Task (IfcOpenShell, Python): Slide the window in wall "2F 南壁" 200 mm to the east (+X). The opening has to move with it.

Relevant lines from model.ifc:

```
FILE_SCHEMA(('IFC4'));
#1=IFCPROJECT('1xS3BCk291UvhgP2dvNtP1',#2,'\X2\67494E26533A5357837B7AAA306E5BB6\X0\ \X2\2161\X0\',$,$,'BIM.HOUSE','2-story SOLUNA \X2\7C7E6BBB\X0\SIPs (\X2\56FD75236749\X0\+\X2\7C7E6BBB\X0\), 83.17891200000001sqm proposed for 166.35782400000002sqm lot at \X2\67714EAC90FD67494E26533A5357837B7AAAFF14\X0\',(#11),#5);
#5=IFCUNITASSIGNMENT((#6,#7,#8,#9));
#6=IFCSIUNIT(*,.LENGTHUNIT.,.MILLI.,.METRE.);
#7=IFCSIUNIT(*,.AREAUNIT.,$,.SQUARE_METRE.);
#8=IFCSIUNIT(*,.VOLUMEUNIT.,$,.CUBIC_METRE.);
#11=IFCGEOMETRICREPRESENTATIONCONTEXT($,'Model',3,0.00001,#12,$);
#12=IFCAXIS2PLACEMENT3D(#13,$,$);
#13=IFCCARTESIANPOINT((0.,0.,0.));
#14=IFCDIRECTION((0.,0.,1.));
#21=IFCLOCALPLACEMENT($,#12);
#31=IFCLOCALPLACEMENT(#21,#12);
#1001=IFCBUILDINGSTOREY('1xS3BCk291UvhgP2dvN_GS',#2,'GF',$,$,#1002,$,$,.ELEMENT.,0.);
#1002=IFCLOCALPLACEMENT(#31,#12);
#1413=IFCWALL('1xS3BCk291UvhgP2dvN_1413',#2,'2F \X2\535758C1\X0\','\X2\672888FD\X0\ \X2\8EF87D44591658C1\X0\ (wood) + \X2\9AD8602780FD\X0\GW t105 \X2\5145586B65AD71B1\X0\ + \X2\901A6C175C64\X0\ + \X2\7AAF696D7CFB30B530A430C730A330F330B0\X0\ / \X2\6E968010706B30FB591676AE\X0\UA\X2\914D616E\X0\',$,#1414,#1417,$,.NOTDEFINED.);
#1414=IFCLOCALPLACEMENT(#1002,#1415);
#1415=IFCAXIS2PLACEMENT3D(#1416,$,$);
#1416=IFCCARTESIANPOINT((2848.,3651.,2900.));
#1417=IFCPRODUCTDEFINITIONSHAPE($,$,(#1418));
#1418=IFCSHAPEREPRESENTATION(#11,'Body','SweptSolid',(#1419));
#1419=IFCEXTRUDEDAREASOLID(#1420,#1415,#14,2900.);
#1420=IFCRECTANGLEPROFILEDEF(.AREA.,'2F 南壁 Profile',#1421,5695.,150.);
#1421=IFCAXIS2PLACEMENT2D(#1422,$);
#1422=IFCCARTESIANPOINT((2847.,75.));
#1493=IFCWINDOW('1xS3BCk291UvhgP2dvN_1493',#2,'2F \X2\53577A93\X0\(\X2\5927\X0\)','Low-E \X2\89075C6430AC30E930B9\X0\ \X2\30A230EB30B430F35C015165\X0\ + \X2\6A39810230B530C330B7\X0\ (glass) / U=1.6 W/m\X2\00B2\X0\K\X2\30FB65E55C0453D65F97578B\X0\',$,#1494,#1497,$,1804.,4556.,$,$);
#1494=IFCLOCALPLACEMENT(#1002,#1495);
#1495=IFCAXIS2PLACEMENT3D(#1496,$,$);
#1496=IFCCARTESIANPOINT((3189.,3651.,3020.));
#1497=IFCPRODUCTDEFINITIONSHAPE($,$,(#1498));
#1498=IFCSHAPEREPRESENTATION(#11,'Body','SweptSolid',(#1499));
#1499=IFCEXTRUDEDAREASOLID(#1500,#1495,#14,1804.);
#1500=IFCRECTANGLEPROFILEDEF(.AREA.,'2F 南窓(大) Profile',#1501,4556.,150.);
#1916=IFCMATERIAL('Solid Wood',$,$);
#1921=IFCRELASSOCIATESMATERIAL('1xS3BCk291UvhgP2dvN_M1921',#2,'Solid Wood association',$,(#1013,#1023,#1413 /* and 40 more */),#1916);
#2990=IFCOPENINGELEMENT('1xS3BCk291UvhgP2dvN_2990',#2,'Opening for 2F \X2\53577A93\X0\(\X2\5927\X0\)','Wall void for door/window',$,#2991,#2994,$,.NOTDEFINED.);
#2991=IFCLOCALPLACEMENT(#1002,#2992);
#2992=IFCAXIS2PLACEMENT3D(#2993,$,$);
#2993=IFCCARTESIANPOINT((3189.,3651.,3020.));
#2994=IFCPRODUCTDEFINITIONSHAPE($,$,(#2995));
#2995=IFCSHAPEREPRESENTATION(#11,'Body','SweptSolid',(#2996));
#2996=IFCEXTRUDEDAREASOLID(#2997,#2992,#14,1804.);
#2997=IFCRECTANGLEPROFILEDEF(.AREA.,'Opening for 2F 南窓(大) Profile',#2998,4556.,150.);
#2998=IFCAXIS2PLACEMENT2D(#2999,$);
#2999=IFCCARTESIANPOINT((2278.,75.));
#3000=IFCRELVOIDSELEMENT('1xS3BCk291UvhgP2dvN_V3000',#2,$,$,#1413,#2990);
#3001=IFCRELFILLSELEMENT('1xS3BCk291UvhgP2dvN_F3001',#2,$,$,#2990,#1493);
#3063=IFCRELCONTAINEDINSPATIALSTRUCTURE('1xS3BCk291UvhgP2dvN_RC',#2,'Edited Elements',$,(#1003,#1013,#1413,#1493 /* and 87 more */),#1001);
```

```python
import ifcopenshell
import ifcopenshell.api.geometry
import ifcopenshell.util.placement

model = ifcopenshell.open("model.ifc")

window = model.by_guid("1xS3BCk291UvhgP2dvN_1493")
opening = window.FillsVoids[0].RelatingOpeningElement
wall = opening.VoidsElements[0].RelatingBuildingElement

wall_matrix = ifcopenshell.util.placement.get_local_placement(wall.ObjectPlacement)
shift = wall_matrix[:3, 0] * 200.0
before = ifcopenshell.util.placement.get_local_placement(window.ObjectPlacement)[:3, 3].copy()

# The window is not placed relative to its opening, so move both.
for product in (opening, window):
    matrix = ifcopenshell.util.placement.get_local_placement(product.ObjectPlacement)
    matrix[:3, 3] += shift
    ifcopenshell.api.geometry.edit_object_placement(model, product=product, matrix=matrix, is_si=False)

after = ifcopenshell.util.placement.get_local_placement(window.ObjectPlacement)[:3, 3]
print("window moved by", (after - before).round(3) + 0.0)

model.write("model_updated.ifc")
```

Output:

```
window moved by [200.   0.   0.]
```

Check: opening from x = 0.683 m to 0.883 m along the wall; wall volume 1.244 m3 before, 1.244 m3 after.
